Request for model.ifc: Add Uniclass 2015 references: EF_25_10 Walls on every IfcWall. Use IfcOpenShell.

First a look at what the model holds.

```python
import ifcopenshell

model = ifcopenshell.open("model.ifc")
print(model.schema)
print("classifications:", [c.Name for c in model.by_type("IfcClassification")])
for ifc_class in ("IfcDoor", "IfcRoof", "IfcStair", "IfcWall", "IfcWindow"):
    print(ifc_class, len(model.by_type(ifc_class)))
```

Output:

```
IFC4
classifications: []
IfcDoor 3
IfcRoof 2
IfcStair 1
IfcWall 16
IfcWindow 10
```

```python
import ifcopenshell
import ifcopenshell.api.classification

model = ifcopenshell.open("model.ifc")

system = ifcopenshell.api.classification.add_classification(model, classification="Uniclass 2015")

codes = {
    "IfcWall": ("EF_25_10", "Walls"),
}
for ifc_class, (code, name) in codes.items():
    products = model.by_type(ifc_class)
    ifcopenshell.api.classification.add_reference(
        model, products=products, classification=system, identification=code, name=name
    )
    print(code, len(products))

model.write("model-out.ifc")
```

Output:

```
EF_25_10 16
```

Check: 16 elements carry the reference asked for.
